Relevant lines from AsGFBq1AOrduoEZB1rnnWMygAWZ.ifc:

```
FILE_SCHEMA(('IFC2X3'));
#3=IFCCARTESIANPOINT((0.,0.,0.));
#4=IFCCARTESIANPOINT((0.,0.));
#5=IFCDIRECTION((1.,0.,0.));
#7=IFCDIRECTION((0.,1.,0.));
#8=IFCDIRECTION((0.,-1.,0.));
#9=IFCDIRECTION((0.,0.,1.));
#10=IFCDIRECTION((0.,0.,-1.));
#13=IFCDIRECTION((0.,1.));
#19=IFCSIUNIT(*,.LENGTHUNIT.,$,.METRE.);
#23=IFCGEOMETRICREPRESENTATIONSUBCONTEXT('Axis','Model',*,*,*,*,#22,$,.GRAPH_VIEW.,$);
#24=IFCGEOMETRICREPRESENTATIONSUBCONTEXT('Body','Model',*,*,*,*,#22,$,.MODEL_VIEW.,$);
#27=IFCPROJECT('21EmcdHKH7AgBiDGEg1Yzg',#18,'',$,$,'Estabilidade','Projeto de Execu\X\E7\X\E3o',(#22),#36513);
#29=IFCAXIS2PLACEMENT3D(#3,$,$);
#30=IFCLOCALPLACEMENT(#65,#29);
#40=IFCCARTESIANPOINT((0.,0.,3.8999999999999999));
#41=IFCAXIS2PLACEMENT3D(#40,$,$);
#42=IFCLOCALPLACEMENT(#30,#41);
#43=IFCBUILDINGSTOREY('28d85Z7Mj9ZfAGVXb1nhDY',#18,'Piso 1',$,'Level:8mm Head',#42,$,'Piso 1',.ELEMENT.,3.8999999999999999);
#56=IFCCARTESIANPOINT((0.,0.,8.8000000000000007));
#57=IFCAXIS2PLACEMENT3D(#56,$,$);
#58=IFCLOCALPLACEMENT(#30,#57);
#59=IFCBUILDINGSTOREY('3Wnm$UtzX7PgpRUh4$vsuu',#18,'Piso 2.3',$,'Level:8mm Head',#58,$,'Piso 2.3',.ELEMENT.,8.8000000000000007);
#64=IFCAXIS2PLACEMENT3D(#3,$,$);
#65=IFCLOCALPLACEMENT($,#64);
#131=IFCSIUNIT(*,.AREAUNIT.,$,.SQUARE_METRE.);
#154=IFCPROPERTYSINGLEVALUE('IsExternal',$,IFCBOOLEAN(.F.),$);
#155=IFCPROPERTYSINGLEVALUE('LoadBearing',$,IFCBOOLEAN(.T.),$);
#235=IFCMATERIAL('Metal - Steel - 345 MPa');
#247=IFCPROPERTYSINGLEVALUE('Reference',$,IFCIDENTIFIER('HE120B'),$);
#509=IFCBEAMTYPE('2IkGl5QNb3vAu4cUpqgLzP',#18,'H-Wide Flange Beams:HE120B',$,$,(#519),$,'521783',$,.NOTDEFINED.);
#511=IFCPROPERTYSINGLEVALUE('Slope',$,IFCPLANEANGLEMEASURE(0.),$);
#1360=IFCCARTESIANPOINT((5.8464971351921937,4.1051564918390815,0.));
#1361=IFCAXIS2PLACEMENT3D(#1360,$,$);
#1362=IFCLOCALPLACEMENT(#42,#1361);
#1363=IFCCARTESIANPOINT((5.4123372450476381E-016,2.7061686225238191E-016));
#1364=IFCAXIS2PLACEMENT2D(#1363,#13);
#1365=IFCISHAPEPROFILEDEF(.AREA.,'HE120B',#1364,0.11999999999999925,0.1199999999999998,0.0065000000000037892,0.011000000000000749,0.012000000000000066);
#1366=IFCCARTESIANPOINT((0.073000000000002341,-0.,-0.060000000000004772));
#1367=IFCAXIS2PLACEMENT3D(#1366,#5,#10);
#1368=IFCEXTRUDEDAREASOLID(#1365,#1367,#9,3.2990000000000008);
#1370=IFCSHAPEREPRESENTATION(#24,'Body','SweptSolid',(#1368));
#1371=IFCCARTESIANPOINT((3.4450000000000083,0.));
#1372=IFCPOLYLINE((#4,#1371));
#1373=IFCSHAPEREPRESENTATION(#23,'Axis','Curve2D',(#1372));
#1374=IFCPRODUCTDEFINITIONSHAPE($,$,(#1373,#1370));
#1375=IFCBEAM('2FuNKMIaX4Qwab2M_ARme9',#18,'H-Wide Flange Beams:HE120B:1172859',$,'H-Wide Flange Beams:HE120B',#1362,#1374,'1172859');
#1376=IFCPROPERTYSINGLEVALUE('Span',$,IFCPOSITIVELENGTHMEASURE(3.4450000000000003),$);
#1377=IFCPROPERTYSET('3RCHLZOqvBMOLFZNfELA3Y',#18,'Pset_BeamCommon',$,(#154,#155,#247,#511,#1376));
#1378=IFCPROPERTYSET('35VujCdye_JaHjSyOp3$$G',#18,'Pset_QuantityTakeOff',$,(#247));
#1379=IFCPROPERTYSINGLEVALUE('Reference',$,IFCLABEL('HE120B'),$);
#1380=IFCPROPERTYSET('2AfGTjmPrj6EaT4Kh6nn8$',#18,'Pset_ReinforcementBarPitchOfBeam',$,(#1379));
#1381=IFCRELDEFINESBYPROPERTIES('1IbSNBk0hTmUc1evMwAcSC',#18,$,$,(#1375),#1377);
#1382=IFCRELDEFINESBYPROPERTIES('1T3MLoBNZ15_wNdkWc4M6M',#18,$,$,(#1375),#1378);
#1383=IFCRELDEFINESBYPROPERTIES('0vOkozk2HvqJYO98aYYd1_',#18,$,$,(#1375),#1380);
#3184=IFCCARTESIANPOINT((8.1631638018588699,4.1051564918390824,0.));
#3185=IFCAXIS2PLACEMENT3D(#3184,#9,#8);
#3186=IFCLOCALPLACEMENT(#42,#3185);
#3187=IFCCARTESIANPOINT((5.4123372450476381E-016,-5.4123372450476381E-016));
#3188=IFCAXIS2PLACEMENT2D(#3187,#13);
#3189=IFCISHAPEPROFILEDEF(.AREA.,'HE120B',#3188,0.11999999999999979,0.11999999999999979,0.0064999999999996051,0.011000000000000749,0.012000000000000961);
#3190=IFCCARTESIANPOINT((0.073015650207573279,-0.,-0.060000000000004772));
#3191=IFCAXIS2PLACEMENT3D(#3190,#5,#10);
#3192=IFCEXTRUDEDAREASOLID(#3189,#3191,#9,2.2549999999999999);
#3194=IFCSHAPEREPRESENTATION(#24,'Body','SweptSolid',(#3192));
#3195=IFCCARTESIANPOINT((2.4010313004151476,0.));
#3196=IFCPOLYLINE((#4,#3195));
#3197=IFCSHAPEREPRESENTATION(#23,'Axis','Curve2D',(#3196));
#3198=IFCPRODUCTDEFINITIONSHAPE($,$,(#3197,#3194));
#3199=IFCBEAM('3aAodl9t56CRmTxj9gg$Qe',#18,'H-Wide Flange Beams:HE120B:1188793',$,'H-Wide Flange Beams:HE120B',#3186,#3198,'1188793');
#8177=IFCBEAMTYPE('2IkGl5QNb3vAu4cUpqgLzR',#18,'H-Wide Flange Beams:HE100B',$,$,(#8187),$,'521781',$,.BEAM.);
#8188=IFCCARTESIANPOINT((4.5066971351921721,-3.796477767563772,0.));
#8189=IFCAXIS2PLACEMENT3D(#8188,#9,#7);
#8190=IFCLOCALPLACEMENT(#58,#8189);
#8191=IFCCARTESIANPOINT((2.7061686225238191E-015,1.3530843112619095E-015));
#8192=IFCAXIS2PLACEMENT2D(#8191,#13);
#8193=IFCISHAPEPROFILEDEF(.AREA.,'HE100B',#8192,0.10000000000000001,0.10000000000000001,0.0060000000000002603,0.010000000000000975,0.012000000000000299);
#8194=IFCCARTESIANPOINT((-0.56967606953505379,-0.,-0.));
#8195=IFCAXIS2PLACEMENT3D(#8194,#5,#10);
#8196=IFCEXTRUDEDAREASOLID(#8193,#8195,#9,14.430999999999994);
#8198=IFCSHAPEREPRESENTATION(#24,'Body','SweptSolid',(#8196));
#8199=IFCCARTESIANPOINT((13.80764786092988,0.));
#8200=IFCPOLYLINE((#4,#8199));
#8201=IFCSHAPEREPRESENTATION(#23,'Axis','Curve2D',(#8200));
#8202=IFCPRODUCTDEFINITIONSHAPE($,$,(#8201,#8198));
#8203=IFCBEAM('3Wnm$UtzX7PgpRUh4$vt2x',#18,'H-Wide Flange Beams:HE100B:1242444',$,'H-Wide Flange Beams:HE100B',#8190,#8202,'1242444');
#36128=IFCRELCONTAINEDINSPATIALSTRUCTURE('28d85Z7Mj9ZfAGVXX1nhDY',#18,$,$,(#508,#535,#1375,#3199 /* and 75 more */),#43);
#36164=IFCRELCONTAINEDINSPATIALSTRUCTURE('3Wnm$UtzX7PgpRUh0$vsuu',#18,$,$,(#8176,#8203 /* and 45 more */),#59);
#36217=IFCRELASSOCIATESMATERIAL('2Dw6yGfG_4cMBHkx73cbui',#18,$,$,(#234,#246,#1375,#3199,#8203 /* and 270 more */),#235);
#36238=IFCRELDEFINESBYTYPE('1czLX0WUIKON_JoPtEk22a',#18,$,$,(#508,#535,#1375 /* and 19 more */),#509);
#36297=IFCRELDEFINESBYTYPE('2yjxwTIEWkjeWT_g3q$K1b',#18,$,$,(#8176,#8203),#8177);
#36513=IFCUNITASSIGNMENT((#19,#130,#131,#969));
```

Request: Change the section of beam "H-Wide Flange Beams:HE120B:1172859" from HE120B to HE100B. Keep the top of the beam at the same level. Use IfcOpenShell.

```python
import ifcopenshell
import ifcopenshell.api.pset
import ifcopenshell.api.type
import ifcopenshell.util.element
import ifcopenshell.util.representation

model = ifcopenshell.open("AsGFBq1AOrduoEZB1rnnWMygAWZ.ifc")

member = model.by_guid("2FuNKMIaX4Qwab2M_ARme9")
source = next(p for p in model.by_type("IfcIShapeProfileDef") if p.ProfileName == "HE100B")

body = ifcopenshell.util.representation.get_representation(member, "Model", "Body")
solid = body.Items[0]
old_profile = solid.SweptArea

# Copy the section's sizes but keep this member's own profile position.
profile = ifcopenshell.util.element.copy(model, source)
# Profiles are centred, so shift by half the change in depth to hold the top.
shift = (old_profile.OverallDepth - profile.OverallDepth) / 2
x, y = old_profile.Position.Location.Coordinates
up = (-1.0, 0.0)  # upwards, in the solid's own plane
location = model.createIfcCartesianPoint((x + up[0] * shift, y + up[1] * shift))
profile.Position = model.createIfcAxis2Placement2D(location, old_profile.Position.RefDirection)
solid.SweptArea = profile
if not model.get_total_inverses(old_profile):
    ifcopenshell.util.element.remove_deep2(model, old_profile)

new_type = model.by_guid("2IkGl5QNb3vAu4cUpqgLzR")
ifcopenshell.api.type.assign_type(
    model, related_objects=[member], relating_type=new_type, should_map_representations=False
)
member.Name = member.Name.replace("HE120B", "HE100B")
member.ObjectType = "H-Wide Flange Beams:HE100B"
pset = model.by_id(ifcopenshell.util.element.get_pset(member, "Pset_BeamCommon", should_inherit=False)["id"])
ifcopenshell.api.pset.edit_pset(model, pset=pset, properties={"Reference": "HE100B"})
pset = model.by_id(ifcopenshell.util.element.get_pset(member, "Pset_QuantityTakeOff", should_inherit=False)["id"])
ifcopenshell.api.pset.edit_pset(model, pset=pset, properties={"Reference": "HE100B"})
pset = model.by_id(ifcopenshell.util.element.get_pset(member, "Pset_ReinforcementBarPitchOfBeam", should_inherit=False)["id"])
ifcopenshell.api.pset.edit_pset(model, pset=pset, properties={"Reference": "HE100B"})

print(solid.SweptArea)

model.write("AsGFBq1AOrduoEZB1rnnWMygAWZ_updated.ifc")
```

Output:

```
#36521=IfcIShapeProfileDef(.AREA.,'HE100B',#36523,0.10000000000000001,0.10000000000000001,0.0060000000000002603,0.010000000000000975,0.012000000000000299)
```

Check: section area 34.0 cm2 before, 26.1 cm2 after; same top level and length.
